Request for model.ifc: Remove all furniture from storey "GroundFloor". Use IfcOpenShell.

First a look at what the model holds.

```python
import ifcopenshell
import ifcopenshell.util.element

model = ifcopenshell.open("model.ifc")
print(model.schema)
storey = next(s for s in model.by_type("IfcBuildingStorey") if s.Name == "GroundFloor")
furniture = [e for e in ifcopenshell.util.element.get_decomposition(storey) if e.is_a("IfcFurnishingElement")]
seen = {}
for e in furniture:
    element_type = ifcopenshell.util.element.get_type(e)
    name = element_type.Name if element_type not in (None, e) else None
    seen[name] = seen.get(name, 0) + 1
for name, count in sorted(seen.items(), key=str):
    print(count, "x", name)
```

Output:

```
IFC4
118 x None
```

```python
import ifcopenshell
import ifcopenshell.api.root
import ifcopenshell.util.element

model = ifcopenshell.open("model.ifc")

storey = next(s for s in model.by_type("IfcBuildingStorey") if s.Name == "GroundFloor")
furniture = [e for e in ifcopenshell.util.element.get_decomposition(storey) if e.is_a("IfcFurnishingElement")]

for e in furniture:
    ifcopenshell.api.root.remove_product(model, product=e)
print(len(furniture), "removed")

model.write("model_rev.ifc")
```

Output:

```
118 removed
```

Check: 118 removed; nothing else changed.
